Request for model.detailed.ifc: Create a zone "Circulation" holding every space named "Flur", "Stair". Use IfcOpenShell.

First a look at what the model holds.

```python
import ifcopenshell

model = ifcopenshell.open("model.detailed.ifc")
print(model.schema)
seen = {}
for space in model.by_type("IfcSpace"):
    seen[space.LongName] = seen.get(space.LongName, 0) + 1
for name, count in sorted(seen.items(), key=str):
    print(count, "x", name)
print("zones:", [z.Name for z in model.by_type("IfcZone")][:20])
```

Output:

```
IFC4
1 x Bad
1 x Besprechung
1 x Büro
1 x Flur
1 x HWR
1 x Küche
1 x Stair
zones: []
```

```python
import ifcopenshell
import ifcopenshell.api.group
import ifcopenshell.api.root

model = ifcopenshell.open("model.detailed.ifc")

names = {"Flur", "Stair"}
spaces = [s for s in model.by_type("IfcSpace") if s.LongName in names]

zone = ifcopenshell.api.root.create_entity(model, ifc_class="IfcZone", name="Circulation")
ifcopenshell.api.group.assign_group(model, products=spaces, group=zone)
print(len(spaces), "spaces in", zone.Name)

model.write("model.detailed_edited.ifc")
```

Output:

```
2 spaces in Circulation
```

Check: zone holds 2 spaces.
